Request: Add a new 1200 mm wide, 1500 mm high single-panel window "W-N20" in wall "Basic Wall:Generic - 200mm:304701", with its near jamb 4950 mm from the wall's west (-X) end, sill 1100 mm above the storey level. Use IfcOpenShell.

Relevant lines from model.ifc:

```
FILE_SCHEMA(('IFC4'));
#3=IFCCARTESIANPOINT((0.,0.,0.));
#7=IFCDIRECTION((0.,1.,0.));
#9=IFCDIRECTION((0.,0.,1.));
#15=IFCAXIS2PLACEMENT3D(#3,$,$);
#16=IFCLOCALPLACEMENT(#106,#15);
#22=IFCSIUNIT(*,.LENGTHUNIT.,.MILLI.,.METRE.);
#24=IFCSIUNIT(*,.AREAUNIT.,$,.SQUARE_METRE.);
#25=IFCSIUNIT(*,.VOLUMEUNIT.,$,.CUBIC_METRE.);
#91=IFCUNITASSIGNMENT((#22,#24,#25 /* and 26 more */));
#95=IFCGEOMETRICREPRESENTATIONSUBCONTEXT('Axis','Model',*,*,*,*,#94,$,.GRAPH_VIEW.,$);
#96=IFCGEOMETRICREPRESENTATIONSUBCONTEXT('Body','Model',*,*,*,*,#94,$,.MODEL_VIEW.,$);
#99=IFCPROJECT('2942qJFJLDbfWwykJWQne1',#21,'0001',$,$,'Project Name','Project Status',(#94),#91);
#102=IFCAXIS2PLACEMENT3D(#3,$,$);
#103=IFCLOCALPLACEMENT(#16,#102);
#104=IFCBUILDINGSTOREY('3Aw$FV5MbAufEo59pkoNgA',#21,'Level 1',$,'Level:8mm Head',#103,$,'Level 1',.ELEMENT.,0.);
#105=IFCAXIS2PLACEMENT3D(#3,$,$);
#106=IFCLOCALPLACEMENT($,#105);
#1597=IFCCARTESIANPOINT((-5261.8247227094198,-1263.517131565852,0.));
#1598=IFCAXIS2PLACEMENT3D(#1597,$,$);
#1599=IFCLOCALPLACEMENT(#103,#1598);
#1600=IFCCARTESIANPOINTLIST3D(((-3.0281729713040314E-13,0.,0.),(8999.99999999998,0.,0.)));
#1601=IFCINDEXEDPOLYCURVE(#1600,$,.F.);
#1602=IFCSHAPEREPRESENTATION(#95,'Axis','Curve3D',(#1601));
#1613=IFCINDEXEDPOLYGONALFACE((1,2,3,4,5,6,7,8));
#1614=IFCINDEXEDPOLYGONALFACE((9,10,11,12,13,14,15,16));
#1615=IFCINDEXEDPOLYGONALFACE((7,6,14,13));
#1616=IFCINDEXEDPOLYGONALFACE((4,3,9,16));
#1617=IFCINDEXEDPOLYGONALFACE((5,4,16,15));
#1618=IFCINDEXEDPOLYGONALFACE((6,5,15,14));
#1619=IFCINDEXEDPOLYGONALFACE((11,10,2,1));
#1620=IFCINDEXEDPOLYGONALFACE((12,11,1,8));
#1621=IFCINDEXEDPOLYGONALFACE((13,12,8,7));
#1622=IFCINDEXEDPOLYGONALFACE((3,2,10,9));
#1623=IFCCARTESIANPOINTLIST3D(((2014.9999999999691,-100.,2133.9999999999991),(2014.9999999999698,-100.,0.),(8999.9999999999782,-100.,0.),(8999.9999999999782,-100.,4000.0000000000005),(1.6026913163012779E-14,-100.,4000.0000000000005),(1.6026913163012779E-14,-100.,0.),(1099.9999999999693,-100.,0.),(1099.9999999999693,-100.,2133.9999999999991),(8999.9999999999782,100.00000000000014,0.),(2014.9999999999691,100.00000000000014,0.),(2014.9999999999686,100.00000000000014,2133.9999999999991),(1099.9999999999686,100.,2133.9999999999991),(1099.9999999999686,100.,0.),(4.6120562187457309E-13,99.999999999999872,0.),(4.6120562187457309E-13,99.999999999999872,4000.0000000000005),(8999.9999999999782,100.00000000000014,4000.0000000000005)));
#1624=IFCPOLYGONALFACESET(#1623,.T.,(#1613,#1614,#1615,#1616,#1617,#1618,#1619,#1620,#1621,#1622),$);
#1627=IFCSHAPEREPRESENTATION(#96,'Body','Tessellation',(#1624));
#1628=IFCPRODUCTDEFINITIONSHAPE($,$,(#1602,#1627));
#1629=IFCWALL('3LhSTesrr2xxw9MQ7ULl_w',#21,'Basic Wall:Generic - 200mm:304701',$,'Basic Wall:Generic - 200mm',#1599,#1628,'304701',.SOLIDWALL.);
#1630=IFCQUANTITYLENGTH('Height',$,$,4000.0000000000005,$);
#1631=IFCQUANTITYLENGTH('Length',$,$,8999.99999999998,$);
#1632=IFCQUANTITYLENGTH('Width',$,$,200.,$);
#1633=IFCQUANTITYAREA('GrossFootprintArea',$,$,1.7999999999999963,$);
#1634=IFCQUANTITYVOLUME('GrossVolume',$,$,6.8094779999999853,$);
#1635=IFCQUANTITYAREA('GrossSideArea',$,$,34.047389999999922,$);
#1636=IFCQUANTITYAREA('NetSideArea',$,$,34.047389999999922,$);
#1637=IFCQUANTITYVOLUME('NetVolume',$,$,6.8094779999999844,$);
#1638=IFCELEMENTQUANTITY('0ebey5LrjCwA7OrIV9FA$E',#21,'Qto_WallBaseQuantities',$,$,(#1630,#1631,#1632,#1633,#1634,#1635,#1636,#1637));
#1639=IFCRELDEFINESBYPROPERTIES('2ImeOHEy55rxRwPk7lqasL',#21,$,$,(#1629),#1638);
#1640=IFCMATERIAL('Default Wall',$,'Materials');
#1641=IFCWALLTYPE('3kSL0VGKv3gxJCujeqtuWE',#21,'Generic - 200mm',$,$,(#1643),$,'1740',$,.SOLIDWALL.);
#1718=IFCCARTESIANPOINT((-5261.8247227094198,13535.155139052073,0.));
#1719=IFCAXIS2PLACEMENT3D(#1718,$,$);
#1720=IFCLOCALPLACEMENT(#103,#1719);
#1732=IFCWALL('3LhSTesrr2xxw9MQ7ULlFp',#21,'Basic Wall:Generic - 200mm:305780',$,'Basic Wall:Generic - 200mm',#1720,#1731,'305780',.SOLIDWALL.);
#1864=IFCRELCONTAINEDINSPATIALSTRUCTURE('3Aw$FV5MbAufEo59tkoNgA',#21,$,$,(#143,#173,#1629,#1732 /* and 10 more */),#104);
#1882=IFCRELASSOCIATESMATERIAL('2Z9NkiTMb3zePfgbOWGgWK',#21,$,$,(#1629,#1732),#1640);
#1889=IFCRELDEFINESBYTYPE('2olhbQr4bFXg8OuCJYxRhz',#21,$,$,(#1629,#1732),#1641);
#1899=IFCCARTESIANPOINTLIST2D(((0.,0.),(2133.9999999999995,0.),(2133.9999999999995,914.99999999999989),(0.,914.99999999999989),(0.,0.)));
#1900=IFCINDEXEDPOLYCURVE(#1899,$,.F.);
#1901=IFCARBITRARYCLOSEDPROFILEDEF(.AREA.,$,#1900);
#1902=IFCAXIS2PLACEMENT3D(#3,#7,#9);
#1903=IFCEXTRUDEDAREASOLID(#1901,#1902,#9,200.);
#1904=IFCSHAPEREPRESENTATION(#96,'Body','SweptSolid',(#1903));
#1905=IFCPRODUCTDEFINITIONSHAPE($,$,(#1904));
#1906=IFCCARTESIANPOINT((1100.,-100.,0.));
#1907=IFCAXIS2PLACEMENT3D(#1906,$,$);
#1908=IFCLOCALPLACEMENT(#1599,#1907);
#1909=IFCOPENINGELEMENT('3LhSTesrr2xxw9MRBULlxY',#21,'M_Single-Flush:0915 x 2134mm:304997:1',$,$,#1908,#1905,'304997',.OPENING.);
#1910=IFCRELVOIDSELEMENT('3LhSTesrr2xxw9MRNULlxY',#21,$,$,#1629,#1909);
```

```python
import numpy as np
import ifcopenshell
import ifcopenshell.api.feature
import ifcopenshell.api.geometry
import ifcopenshell.api.pset
import ifcopenshell.api.root
import ifcopenshell.api.spatial
import ifcopenshell.geom
import ifcopenshell.util.element
import ifcopenshell.util.placement
import ifcopenshell.util.representation
import ifcopenshell.util.shape
import ifcopenshell.util.unit

model = ifcopenshell.open("model.ifc")
unit_scale = ifcopenshell.util.unit.calculate_unit_scale(model)
area_scale = ifcopenshell.util.unit.calculate_unit_scale(model, "AREAUNIT")
volume_scale = ifcopenshell.util.unit.calculate_unit_scale(model, "VOLUMEUNIT")
settings = ifcopenshell.geom.settings()


def volume(element):
    """Net volume in cubic metres, openings subtracted."""
    shape = ifcopenshell.geom.create_shape(settings, element)
    return ifcopenshell.util.shape.get_volume(shape.geometry)


wall = model.by_id(1629)
storey = ifcopenshell.util.element.get_container(wall, ifc_class="IfcBuildingStorey")
context = ifcopenshell.util.representation.get_context(model, "Model", "Body", "MODEL_VIEW")
before = volume(wall)

width, height, from_end, sill = 1.2, 1.5, 4.95, 1.1  # metres

# The wall runs along its own X axis, and the end named is its -X end.
wall_shape = ifcopenshell.geom.create_shape(settings, wall)
x, y, z = ifcopenshell.util.shape.get_vertices(wall_shape.geometry).T
start = x.min() + from_end
face, thickness = float(y.min()), float(y.max() - y.min())
wall_matrix = ifcopenshell.util.placement.get_local_placement(wall.ObjectPlacement)
level = ifcopenshell.util.placement.get_local_placement(storey.ObjectPlacement)[2, 3]


def in_wall(x, y):
    """Placement at x, y metres in the wall's axes, at sill height."""
    matrix = wall_matrix.copy()
    matrix[:, 3] = wall_matrix @ np.array([x / unit_scale, y / unit_scale, 0.0, 1.0])
    matrix[2, 3] = level + sill / unit_scale
    return matrix


# Opening: a box that overshoots both wall faces by 50 mm.
opening = ifcopenshell.api.root.create_entity(model, ifc_class="IfcOpeningElement", predefined_type="OPENING")
box = ifcopenshell.api.geometry.add_wall_representation(
    model, context=context, length=width, height=height, thickness=thickness + 0.1
)
ifcopenshell.api.geometry.assign_representation(model, product=opening, representation=box)
ifcopenshell.api.geometry.edit_object_placement(model, product=opening, matrix=in_wall(start, face - 0.05), is_si=False)
ifcopenshell.api.feature.add_feature(model, feature=opening, element=wall)

window = ifcopenshell.api.root.create_entity(model, ifc_class="IfcWindow", name="W-N20", predefined_type="WINDOW")
window.OverallWidth, window.OverallHeight = width / unit_scale, height / unit_scale
window.PartitioningType = "SINGLE_PANEL"
body = ifcopenshell.api.geometry.add_window_representation(
    model,
    context=context,
    overall_width=window.OverallWidth,
    overall_height=window.OverallHeight,
    partition_type="SINGLE_PANEL",
)
ifcopenshell.api.geometry.assign_representation(model, product=window, representation=body)
ifcopenshell.api.spatial.assign_container(model, products=[window], relating_structure=storey)
ifcopenshell.api.feature.add_filling(model, opening=opening, element=window)

# Centre the window in the wall's thickness.
ifcopenshell.api.geometry.edit_object_placement(model, product=window, matrix=in_wall(start, face), is_si=False)
window_shape = ifcopenshell.geom.create_shape(settings, window)
depth = ifcopenshell.util.shape.get_vertices(window_shape.geometry)[:, 1]
offset = face + thickness / 2 - (depth.min() + depth.max()) / 2
ifcopenshell.api.geometry.edit_object_placement(model, product=window, matrix=in_wall(start, offset), is_si=False)

after = volume(wall)

# Update the wall's stored quantities.
qto = model.by_id(ifcopenshell.util.element.get_pset(wall, "Qto_WallBaseQuantities", should_inherit=False)["id"])
ifcopenshell.api.pset.edit_qto(model, qto=qto, properties={
    "NetSideArea": after / thickness / area_scale,
    "NetVolume": after / volume_scale,
})

print(f"wall volume {before:.3f} -> {after:.3f} m3")

model.write("model_v2.ifc")
```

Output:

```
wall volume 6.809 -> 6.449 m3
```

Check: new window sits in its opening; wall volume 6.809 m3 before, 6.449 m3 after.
